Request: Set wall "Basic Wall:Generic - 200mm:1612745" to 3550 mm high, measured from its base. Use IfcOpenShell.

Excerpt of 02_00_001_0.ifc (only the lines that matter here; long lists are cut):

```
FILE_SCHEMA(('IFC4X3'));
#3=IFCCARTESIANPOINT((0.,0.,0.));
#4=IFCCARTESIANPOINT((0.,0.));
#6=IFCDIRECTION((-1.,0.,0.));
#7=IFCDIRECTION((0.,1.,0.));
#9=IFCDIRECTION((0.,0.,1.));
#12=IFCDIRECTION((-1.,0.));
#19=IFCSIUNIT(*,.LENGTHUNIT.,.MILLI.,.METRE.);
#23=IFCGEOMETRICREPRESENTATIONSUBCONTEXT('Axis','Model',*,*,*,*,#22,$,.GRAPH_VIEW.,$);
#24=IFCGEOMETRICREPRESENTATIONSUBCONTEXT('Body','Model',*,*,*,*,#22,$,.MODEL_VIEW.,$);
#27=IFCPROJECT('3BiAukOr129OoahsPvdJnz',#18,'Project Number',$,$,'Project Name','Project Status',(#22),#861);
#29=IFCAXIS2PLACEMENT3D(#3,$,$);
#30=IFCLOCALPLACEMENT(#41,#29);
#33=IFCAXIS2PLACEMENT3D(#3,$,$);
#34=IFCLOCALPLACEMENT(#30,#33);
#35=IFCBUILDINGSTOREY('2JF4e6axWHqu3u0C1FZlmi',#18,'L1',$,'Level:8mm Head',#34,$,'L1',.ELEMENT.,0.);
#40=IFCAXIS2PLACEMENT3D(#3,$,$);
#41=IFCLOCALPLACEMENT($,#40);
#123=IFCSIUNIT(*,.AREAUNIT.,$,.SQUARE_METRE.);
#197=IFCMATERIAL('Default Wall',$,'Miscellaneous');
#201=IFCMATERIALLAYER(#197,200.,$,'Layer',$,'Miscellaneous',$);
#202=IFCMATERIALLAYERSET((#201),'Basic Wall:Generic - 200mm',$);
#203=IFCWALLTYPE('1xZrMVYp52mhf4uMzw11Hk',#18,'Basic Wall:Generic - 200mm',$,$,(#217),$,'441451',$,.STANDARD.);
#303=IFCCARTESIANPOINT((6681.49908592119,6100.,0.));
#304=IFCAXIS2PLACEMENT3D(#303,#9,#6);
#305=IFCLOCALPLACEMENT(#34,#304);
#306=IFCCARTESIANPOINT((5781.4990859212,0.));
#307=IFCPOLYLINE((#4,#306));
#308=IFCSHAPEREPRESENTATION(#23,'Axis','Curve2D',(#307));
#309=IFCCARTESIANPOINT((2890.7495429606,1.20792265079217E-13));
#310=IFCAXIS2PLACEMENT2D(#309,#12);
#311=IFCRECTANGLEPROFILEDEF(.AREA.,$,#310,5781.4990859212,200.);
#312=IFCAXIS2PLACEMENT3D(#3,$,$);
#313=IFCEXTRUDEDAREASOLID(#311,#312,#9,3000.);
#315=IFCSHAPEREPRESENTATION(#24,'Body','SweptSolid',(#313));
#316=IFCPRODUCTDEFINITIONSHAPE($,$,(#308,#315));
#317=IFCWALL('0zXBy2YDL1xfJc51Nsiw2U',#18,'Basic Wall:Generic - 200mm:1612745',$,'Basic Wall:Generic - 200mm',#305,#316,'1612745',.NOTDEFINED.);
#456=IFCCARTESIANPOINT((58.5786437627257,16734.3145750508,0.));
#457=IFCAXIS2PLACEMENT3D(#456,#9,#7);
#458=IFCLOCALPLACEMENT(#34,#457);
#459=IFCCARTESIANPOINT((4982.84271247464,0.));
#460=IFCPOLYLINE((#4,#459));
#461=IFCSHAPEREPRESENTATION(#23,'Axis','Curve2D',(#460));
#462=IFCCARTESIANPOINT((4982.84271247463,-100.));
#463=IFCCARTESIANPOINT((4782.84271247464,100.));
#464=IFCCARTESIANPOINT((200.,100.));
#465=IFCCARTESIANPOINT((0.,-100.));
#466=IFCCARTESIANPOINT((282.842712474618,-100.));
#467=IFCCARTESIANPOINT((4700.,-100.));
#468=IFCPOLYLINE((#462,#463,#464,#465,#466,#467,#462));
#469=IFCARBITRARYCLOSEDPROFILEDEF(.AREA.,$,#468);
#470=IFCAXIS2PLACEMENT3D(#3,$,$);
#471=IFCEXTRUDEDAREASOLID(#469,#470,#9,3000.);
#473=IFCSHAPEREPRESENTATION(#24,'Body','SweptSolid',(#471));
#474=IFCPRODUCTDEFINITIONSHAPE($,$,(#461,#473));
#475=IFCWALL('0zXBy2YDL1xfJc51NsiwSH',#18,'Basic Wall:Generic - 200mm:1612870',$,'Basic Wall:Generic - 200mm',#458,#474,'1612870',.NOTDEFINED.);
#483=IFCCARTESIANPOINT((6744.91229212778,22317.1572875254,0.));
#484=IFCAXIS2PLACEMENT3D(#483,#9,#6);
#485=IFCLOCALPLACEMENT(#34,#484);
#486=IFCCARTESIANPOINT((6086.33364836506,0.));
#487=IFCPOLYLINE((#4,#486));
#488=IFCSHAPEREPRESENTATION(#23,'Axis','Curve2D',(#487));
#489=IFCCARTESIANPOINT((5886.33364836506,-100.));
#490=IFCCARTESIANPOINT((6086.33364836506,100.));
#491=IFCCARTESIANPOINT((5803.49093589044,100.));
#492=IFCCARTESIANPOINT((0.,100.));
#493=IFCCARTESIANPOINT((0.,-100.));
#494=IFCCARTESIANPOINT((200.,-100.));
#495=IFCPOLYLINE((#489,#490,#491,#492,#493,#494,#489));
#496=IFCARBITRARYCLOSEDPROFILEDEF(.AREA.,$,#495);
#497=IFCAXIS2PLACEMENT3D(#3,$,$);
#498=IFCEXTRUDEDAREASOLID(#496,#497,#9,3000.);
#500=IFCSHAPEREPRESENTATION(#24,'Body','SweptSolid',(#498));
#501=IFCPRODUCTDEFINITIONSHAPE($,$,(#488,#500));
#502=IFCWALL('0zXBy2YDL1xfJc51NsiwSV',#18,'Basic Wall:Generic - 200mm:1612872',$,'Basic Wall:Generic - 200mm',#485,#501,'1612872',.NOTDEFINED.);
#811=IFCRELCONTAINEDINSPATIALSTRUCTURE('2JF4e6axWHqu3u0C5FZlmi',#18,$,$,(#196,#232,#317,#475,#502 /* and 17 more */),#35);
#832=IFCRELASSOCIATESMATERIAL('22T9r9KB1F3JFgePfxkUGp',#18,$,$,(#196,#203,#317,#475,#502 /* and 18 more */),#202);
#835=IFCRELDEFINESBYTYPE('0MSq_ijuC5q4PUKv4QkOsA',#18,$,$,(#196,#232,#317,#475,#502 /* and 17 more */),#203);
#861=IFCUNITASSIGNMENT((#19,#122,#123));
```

```python
import ifcopenshell
import ifcopenshell.geom
import ifcopenshell.util.representation
import ifcopenshell.util.shape

model = ifcopenshell.open("02_00_001_0.ifc")
settings = ifcopenshell.geom.settings()


def volume(element):
    """Net volume in cubic metres, openings subtracted."""
    shape = ifcopenshell.geom.create_shape(settings, element)
    return ifcopenshell.util.shape.get_volume(shape.geometry)


wall = model.by_id(317)
before = volume(wall)

body = ifcopenshell.util.representation.get_representation(wall, "Model", "Body")
solid = body.Items[0]
old_height = solid.Depth
solid.Depth = 3550.0
after = volume(wall)

print(f"height {old_height:g} -> {solid.Depth:g}, volume {before:.3f} -> {after:.3f} m3")

model.write("02_00_001_0-out.ifc")
```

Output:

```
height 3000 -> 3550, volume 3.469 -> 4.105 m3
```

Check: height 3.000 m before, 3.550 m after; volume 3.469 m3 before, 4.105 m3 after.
